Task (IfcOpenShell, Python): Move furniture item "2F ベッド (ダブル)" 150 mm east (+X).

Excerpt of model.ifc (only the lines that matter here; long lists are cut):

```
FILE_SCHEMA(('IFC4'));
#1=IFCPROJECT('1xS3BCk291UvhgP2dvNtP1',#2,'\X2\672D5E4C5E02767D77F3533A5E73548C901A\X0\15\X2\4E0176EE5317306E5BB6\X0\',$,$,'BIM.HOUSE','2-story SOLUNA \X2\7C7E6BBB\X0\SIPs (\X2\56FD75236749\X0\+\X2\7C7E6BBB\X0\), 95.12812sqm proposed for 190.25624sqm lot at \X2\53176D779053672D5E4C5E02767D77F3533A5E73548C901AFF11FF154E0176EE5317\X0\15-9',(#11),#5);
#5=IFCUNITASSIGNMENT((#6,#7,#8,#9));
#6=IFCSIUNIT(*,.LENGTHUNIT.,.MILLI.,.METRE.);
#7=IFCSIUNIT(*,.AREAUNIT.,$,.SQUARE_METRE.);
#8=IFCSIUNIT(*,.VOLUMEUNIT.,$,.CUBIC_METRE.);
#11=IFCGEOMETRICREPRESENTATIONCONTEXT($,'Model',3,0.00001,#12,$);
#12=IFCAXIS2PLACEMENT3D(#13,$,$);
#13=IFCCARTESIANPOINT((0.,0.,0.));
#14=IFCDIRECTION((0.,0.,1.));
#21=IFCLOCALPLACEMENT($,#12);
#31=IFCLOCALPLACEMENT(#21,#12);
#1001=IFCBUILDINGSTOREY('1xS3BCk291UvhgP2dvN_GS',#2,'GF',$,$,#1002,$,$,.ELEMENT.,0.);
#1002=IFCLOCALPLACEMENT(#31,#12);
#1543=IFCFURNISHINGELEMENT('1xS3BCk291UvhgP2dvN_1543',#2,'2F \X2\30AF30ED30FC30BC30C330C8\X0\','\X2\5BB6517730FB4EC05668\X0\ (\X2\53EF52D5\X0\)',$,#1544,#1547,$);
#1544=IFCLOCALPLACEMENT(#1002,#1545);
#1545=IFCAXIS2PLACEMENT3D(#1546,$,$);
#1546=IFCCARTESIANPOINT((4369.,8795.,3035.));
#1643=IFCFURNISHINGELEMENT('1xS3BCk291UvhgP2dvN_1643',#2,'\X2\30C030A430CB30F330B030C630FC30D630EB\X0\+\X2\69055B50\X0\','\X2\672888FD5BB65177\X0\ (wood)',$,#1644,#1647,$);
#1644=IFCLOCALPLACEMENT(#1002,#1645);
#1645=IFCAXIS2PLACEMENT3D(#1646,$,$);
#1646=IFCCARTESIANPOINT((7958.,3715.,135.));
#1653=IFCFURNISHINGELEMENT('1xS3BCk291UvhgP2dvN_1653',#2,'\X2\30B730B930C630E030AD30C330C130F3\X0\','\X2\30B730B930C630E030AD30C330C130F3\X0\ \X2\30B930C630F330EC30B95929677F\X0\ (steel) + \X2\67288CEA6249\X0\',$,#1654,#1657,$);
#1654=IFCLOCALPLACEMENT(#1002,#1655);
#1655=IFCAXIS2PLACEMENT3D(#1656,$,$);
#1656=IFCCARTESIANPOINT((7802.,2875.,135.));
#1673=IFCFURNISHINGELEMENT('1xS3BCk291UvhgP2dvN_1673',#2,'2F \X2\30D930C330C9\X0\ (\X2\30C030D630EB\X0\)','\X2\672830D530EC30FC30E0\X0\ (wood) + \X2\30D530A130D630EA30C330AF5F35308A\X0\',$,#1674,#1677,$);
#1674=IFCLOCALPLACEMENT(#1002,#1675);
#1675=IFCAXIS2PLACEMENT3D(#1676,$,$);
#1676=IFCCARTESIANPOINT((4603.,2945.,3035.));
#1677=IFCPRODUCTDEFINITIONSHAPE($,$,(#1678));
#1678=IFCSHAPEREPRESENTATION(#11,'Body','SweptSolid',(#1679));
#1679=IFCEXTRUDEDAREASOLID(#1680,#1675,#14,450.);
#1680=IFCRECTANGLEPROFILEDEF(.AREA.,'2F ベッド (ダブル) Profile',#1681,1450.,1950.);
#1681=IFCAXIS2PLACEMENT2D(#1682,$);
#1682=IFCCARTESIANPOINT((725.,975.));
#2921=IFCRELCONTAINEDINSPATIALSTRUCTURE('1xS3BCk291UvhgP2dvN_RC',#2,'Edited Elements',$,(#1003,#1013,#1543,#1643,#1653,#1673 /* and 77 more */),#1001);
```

```python
import ifcopenshell
import ifcopenshell.api.geometry
import ifcopenshell.util.placement
import ifcopenshell.util.unit

model = ifcopenshell.open("model.ifc")
unit_scale = ifcopenshell.util.unit.calculate_unit_scale(model)

item = model.by_guid("1xS3BCk291UvhgP2dvN_1673")
matrix = ifcopenshell.util.placement.get_local_placement(item.ObjectPlacement)
matrix[0, 3] += 0.15 / unit_scale
ifcopenshell.api.geometry.edit_object_placement(model, product=item, matrix=matrix, is_si=False)

print(ifcopenshell.util.placement.get_local_placement(item.ObjectPlacement).round(3) + 0.0)

model.write("model_edited.ifc")
```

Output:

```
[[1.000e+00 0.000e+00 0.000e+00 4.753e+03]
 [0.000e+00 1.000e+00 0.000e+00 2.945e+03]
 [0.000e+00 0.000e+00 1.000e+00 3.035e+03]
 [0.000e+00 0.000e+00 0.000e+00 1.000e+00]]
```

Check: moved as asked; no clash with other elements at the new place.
